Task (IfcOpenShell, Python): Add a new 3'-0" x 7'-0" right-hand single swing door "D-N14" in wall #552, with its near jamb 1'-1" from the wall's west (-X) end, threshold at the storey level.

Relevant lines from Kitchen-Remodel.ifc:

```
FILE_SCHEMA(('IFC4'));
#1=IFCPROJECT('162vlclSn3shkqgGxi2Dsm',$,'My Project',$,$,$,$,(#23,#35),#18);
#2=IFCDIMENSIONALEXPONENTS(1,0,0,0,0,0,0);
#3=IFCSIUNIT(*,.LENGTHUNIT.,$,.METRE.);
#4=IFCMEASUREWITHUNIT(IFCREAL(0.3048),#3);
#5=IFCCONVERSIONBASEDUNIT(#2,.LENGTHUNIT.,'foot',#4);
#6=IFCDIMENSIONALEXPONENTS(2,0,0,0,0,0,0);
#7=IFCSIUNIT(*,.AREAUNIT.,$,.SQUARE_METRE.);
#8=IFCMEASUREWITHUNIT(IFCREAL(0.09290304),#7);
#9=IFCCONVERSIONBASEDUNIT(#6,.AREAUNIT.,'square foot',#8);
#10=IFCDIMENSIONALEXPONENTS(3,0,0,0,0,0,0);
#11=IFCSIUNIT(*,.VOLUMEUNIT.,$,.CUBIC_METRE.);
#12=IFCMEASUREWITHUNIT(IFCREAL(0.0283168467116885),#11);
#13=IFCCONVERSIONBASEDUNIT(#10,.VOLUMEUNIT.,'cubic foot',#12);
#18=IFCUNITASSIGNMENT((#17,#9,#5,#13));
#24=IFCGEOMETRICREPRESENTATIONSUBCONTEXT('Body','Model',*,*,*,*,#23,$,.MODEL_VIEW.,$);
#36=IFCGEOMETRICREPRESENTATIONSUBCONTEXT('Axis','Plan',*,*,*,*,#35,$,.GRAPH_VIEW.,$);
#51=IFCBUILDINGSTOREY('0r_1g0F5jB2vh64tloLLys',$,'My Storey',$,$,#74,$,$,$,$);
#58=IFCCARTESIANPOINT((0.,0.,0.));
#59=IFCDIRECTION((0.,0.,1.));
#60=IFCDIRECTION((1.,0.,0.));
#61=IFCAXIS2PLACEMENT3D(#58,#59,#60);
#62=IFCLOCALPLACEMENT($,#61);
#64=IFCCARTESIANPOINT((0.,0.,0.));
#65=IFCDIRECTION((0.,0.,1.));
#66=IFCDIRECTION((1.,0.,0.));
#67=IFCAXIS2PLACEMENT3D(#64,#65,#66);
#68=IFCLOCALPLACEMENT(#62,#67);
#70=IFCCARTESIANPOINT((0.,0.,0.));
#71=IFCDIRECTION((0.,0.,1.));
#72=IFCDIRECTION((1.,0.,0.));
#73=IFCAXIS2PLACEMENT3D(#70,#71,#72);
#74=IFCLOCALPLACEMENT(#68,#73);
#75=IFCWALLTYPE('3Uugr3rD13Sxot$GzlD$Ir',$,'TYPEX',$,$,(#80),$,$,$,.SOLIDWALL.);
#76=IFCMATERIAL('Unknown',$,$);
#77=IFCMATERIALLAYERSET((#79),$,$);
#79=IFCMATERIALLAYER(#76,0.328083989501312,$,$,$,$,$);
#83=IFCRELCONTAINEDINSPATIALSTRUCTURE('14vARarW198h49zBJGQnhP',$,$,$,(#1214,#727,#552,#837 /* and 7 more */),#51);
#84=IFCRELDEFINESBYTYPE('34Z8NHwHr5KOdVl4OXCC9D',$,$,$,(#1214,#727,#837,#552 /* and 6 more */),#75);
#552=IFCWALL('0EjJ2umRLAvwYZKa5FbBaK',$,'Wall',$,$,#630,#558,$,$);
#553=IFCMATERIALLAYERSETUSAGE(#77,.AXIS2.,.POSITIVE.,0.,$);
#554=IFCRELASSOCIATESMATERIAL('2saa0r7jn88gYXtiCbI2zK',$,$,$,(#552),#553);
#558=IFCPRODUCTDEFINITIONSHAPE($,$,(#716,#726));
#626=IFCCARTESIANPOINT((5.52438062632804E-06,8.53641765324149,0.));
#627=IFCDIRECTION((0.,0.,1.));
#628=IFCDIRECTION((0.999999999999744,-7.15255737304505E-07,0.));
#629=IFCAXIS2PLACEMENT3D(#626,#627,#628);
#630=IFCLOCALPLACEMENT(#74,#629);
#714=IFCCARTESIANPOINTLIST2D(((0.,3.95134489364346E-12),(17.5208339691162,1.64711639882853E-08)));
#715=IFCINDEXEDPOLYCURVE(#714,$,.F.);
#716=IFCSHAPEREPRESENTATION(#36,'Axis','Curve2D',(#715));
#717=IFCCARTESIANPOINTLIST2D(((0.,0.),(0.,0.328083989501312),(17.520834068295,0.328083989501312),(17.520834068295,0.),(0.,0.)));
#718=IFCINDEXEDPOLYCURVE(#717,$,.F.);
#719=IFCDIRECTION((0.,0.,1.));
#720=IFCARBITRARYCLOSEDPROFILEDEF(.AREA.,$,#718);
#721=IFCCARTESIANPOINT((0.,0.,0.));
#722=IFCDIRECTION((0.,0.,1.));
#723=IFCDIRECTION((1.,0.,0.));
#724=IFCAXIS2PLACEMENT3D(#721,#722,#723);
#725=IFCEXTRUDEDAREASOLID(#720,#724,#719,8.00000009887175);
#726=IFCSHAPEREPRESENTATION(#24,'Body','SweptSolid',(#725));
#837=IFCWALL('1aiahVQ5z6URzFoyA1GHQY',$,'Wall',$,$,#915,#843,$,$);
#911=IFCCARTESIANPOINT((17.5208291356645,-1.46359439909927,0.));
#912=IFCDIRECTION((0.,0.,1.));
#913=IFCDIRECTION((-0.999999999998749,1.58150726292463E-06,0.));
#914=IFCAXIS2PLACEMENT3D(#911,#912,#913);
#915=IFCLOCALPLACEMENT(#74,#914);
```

```python
import numpy as np
import ifcopenshell
import ifcopenshell.api.feature
import ifcopenshell.api.geometry
import ifcopenshell.api.root
import ifcopenshell.api.spatial
import ifcopenshell.geom
import ifcopenshell.util.element
import ifcopenshell.util.placement
import ifcopenshell.util.representation
import ifcopenshell.util.shape
import ifcopenshell.util.unit

model = ifcopenshell.open("Kitchen-Remodel.ifc")
unit_scale = ifcopenshell.util.unit.calculate_unit_scale(model)
settings = ifcopenshell.geom.settings()


def volume(element):
    """Net volume in cubic metres, openings subtracted."""
    shape = ifcopenshell.geom.create_shape(settings, element)
    return ifcopenshell.util.shape.get_volume(shape.geometry)


wall = model.by_guid("0EjJ2umRLAvwYZKa5FbBaK")
storey = ifcopenshell.util.element.get_container(wall, ifc_class="IfcBuildingStorey")
context = ifcopenshell.util.representation.get_context(model, "Model", "Body", "MODEL_VIEW")
before = volume(wall)

width, height, from_end, sill = 0.9144, 2.1336, 0.3302, 0.0  # metres

# The wall runs along its own X axis, and the end named is its -X end.
wall_shape = ifcopenshell.geom.create_shape(settings, wall)
x, y, z = ifcopenshell.util.shape.get_vertices(wall_shape.geometry).T
start = x.min() + from_end
face, thickness = float(y.min()), float(y.max() - y.min())
wall_matrix = ifcopenshell.util.placement.get_local_placement(wall.ObjectPlacement)
level = ifcopenshell.util.placement.get_local_placement(storey.ObjectPlacement)[2, 3]


def in_wall(x, y):
    """Placement at x, y metres in the wall's axes, at sill height."""
    matrix = wall_matrix.copy()
    matrix[:, 3] = wall_matrix @ np.array([x / unit_scale, y / unit_scale, 0.0, 1.0])
    matrix[2, 3] = level + sill / unit_scale
    return matrix


# Opening: a box that overshoots both wall faces by 50 mm.
opening = ifcopenshell.api.root.create_entity(model, ifc_class="IfcOpeningElement", predefined_type="OPENING")
box = ifcopenshell.api.geometry.add_wall_representation(
    model, context=context, length=width, height=height, thickness=thickness + 0.1
)
ifcopenshell.api.geometry.assign_representation(model, product=opening, representation=box)
ifcopenshell.api.geometry.edit_object_placement(model, product=opening, matrix=in_wall(start, face - 0.05), is_si=False)
ifcopenshell.api.feature.add_feature(model, feature=opening, element=wall)

door = ifcopenshell.api.root.create_entity(model, ifc_class="IfcDoor", name="D-N14", predefined_type="DOOR")
door.OverallWidth, door.OverallHeight = width / unit_scale, height / unit_scale
door.OperationType = "SINGLE_SWING_RIGHT"
body = ifcopenshell.api.geometry.add_door_representation(
    model,
    context=context,
    overall_width=door.OverallWidth,
    overall_height=door.OverallHeight,
    operation_type="SINGLE_SWING_RIGHT",
    lining_properties={"LiningDepth": thickness / unit_scale, "ThresholdDepth": thickness / unit_scale},
)
ifcopenshell.api.geometry.assign_representation(model, product=door, representation=body)
ifcopenshell.api.spatial.assign_container(model, products=[door], relating_structure=storey)
ifcopenshell.api.feature.add_filling(model, opening=opening, element=door)

# The lining spans the wall, so the door starts at the wall face.
ifcopenshell.api.geometry.edit_object_placement(model, product=door, matrix=in_wall(start, face), is_si=False)

after = volume(wall)

print(f"wall volume {before:.3f} -> {after:.3f} m3")

model.write("Kitchen-Remodel_rev.ifc")
```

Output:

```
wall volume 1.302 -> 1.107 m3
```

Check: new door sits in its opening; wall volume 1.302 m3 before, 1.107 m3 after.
